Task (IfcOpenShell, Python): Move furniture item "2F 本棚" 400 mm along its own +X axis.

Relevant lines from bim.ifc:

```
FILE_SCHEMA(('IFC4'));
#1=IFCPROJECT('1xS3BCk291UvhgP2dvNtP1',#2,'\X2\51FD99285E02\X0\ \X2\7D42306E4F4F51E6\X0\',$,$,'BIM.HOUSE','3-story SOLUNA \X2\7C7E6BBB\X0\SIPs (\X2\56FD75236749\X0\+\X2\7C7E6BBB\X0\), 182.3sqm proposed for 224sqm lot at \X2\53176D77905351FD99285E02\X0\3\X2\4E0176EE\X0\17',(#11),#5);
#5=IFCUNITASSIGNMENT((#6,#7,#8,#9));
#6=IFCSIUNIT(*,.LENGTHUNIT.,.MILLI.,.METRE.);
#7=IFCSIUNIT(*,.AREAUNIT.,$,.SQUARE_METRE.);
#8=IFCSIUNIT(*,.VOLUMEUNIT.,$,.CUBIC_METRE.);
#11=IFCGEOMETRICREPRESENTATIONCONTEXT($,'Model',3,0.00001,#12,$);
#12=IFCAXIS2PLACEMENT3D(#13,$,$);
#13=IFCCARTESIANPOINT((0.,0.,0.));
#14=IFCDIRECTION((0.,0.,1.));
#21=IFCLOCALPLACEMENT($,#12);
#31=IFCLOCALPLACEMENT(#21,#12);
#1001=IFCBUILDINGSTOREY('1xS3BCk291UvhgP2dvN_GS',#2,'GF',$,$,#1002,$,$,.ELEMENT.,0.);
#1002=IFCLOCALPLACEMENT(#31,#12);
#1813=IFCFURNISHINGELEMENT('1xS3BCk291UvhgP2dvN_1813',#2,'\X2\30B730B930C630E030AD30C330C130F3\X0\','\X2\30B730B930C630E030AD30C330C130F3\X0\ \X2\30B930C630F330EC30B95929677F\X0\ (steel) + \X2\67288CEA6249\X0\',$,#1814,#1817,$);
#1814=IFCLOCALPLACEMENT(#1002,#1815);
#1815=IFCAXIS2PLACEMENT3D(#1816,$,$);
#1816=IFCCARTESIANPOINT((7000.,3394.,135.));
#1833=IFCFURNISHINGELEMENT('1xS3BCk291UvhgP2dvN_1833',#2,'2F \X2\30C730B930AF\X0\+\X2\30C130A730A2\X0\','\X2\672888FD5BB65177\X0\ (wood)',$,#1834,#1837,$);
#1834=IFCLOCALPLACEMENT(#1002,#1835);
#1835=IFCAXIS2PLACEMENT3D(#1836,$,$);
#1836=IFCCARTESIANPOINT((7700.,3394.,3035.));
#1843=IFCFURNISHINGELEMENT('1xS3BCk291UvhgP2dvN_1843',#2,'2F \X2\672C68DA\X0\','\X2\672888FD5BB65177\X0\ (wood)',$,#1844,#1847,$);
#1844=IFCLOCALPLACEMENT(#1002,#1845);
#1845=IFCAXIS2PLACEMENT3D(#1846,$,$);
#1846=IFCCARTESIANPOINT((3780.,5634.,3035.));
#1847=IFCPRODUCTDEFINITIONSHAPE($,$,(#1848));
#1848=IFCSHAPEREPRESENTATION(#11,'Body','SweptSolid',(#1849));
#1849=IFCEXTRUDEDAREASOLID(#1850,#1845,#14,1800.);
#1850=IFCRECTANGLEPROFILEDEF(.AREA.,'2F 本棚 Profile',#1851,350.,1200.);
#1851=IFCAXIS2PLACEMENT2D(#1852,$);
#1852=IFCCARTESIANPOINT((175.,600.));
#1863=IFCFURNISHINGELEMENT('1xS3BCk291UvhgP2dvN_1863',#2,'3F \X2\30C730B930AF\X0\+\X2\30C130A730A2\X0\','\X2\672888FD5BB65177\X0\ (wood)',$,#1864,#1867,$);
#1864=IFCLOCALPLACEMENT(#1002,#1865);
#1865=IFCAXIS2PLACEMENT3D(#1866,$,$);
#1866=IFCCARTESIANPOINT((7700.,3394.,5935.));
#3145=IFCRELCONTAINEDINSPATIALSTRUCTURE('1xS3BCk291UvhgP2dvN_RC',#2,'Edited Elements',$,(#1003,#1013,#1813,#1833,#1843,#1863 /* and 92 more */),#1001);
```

```python
import ifcopenshell
import ifcopenshell.api.geometry
import ifcopenshell.util.placement

model = ifcopenshell.open("bim.ifc")

item = model.by_guid("1xS3BCk291UvhgP2dvN_1843")
matrix = ifcopenshell.util.placement.get_local_placement(item.ObjectPlacement)
matrix[:3, 3] += matrix[:3, 0] * 400.0
ifcopenshell.api.geometry.edit_object_placement(model, product=item, matrix=matrix, is_si=False)

print(ifcopenshell.util.placement.get_local_placement(item.ObjectPlacement).round(3) + 0.0)

model.write("bim_updated.ifc")
```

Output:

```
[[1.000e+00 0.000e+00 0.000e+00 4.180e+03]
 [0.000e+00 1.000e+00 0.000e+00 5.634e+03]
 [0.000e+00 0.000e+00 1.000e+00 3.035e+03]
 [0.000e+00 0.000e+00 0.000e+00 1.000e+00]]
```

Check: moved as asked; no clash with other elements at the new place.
